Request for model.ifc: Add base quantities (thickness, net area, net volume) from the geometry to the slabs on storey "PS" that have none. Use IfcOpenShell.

First a look at what the model holds.

```python
import ifcopenshell
import ifcopenshell.util.element
import ifcopenshell.util.unit

model = ifcopenshell.open("model.ifc")
print(model.schema)
for unit_type in ("LENGTHUNIT", "AREAUNIT", "VOLUMEUNIT"):
    print(unit_type, ifcopenshell.util.unit.calculate_unit_scale(model, unit_type))
storey = next(s for s in model.by_type("IfcBuildingStorey") if s.Name == "PS")
slabs = [e for e in ifcopenshell.util.element.get_decomposition(storey) if e.is_a("IfcSlab")]
for e in sorted(slabs, key=lambda e: e.id()):
    print(e.id(), e.is_a(), e.Name, list(ifcopenshell.util.element.get_psets(e, qtos_only=True)), sep=" | ")
```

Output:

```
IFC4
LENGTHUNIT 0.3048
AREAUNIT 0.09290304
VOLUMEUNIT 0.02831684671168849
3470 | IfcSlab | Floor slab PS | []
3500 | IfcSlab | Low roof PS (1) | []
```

```python
import ifcopenshell
import ifcopenshell.api.pset
import ifcopenshell.geom
import ifcopenshell.util.element
import ifcopenshell.util.shape
import ifcopenshell.util.unit

model = ifcopenshell.open("model.ifc")
unit_scale = ifcopenshell.util.unit.calculate_unit_scale(model)
area_scale = ifcopenshell.util.unit.calculate_unit_scale(model, "AREAUNIT")
volume_scale = ifcopenshell.util.unit.calculate_unit_scale(model, "VOLUMEUNIT")
settings = ifcopenshell.geom.settings()

storey = next(s for s in model.by_type("IfcBuildingStorey") if s.Name == "PS")
slabs = [e for e in ifcopenshell.util.element.get_decomposition(storey) if e.is_a("IfcSlab")]

for e in sorted(slabs, key=lambda e: e.id()):
    if ifcopenshell.util.element.get_psets(e, qtos_only=True, should_inherit=False):
        continue
    # Geometry comes back in metres, in the element's own axes.
    shape = ifcopenshell.geom.create_shape(settings, e)
    values = {
        "Width": ifcopenshell.util.shape.get_z(shape.geometry) / unit_scale,
        "NetArea": ifcopenshell.util.shape.get_footprint_area(shape.geometry) / area_scale,
        "NetVolume": ifcopenshell.util.shape.get_volume(shape.geometry) / volume_scale,
    }
    qto = ifcopenshell.api.pset.add_qto(model, product=e, name="Qto_SlabBaseQuantities")
    ifcopenshell.api.pset.edit_qto(model, qto=qto, properties=values)
    print(e.id(), {k: round(v, 3) for k, v in values.items()})

model.write("model_v2.ifc")
```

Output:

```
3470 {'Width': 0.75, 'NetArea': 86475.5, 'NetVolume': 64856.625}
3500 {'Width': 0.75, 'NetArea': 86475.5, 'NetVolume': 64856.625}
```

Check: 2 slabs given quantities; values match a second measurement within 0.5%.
